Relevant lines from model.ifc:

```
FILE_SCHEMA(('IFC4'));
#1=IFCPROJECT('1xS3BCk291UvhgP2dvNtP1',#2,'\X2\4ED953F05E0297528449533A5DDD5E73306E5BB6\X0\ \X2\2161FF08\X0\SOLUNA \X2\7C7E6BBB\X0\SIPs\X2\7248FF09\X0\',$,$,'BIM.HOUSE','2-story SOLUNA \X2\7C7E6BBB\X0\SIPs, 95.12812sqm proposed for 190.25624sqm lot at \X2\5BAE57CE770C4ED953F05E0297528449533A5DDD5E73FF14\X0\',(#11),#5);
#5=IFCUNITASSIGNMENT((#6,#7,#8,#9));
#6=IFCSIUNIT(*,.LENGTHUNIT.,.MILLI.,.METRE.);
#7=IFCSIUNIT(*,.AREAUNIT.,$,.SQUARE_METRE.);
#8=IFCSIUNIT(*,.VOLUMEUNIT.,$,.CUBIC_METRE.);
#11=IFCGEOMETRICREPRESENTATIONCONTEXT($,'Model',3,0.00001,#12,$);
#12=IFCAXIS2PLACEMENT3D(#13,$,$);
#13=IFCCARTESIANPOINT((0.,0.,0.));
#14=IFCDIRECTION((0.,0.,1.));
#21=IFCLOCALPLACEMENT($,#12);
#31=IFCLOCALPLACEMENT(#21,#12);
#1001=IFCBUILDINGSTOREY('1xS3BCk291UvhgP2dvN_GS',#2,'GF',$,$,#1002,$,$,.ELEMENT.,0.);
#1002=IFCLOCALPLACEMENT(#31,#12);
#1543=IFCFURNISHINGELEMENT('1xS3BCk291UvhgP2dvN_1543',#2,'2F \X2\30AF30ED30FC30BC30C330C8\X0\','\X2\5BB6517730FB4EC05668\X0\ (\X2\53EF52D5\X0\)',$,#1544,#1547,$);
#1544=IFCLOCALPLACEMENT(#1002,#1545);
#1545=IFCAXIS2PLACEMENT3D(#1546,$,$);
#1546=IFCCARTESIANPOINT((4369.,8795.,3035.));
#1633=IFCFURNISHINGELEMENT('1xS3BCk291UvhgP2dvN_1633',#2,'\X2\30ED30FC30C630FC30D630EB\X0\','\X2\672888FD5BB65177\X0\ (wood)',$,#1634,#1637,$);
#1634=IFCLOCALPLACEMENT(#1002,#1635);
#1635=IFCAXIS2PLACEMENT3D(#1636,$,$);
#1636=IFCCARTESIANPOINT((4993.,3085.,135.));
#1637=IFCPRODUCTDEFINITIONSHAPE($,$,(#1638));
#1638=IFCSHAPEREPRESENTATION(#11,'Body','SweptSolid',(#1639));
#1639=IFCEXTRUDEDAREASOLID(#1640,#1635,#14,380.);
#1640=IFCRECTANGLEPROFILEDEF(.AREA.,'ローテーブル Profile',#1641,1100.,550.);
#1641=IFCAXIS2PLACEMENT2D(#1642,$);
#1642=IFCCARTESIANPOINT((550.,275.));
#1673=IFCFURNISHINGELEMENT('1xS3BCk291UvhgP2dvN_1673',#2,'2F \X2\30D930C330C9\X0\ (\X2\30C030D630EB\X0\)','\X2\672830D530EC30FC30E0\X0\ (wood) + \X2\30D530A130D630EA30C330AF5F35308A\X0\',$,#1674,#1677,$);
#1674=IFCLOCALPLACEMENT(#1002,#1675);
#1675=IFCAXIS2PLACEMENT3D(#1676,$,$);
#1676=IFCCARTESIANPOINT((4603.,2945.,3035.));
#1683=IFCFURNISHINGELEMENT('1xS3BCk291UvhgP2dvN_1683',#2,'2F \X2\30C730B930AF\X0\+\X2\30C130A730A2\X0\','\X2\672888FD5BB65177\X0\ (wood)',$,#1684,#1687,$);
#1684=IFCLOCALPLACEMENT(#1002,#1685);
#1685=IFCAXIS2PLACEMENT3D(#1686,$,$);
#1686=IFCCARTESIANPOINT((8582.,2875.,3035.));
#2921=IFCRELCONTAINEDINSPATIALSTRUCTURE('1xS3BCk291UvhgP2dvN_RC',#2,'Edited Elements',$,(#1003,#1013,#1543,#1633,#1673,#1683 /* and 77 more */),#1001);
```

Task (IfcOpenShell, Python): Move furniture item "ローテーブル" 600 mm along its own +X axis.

```python
import ifcopenshell
import ifcopenshell.api.geometry
import ifcopenshell.util.placement

model = ifcopenshell.open("model.ifc")

item = model.by_guid("1xS3BCk291UvhgP2dvN_1633")
matrix = ifcopenshell.util.placement.get_local_placement(item.ObjectPlacement)
matrix[:3, 3] += matrix[:3, 0] * 600.0
ifcopenshell.api.geometry.edit_object_placement(model, product=item, matrix=matrix, is_si=False)

print(ifcopenshell.util.placement.get_local_placement(item.ObjectPlacement).round(3) + 0.0)

model.write("model_v2.ifc")
```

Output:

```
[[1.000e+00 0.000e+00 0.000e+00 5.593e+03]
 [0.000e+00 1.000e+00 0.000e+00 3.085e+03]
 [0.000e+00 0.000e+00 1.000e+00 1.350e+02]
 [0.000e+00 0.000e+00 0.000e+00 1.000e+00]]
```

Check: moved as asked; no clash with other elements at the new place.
